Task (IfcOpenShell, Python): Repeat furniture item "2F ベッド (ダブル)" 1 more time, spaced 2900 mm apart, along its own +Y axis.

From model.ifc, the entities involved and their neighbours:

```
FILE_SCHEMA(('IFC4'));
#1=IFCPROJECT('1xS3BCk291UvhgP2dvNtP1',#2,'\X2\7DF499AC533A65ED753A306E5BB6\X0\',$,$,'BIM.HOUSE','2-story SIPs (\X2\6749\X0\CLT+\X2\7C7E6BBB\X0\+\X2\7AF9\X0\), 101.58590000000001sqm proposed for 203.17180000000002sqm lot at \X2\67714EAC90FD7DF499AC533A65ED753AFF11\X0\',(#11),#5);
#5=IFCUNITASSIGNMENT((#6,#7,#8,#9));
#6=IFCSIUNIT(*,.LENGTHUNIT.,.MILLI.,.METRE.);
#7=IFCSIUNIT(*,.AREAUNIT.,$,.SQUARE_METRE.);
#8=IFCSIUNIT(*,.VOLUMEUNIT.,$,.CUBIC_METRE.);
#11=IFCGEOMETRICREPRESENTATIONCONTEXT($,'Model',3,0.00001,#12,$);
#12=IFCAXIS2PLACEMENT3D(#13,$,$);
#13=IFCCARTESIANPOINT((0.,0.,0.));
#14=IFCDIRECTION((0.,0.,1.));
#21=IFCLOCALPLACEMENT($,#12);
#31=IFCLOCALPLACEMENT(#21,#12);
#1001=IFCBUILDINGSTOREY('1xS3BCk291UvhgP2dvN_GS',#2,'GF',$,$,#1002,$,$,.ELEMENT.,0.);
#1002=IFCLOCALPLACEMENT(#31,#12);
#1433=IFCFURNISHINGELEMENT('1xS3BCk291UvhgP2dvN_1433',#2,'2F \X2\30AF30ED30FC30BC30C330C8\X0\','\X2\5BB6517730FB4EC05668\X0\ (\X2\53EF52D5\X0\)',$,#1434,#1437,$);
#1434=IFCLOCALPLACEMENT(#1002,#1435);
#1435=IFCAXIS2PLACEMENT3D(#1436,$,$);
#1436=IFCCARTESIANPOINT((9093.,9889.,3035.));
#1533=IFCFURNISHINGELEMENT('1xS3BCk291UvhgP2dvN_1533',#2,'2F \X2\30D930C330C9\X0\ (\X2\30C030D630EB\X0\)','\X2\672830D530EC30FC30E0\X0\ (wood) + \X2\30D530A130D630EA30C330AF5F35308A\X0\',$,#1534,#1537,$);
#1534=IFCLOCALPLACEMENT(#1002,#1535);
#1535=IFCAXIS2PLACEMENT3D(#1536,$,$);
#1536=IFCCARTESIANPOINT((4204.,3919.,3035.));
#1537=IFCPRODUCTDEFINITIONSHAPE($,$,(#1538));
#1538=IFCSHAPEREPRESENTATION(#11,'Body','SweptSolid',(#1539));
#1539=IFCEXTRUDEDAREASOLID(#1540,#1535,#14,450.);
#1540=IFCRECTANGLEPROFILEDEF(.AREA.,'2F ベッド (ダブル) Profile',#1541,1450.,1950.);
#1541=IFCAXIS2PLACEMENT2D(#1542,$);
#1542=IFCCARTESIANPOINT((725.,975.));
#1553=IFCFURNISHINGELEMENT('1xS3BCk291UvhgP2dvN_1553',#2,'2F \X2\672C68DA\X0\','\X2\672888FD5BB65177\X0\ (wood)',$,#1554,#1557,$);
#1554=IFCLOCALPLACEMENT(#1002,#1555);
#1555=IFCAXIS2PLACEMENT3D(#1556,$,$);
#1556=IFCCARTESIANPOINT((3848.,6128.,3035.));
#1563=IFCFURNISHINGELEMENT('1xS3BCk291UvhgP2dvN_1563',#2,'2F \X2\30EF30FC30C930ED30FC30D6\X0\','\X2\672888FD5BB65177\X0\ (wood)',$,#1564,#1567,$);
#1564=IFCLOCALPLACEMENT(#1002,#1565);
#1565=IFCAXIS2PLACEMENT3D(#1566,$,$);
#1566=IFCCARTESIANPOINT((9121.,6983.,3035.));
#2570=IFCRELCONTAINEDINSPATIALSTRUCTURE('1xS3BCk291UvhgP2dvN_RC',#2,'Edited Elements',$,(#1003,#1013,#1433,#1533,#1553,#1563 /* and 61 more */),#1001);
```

```python
import ifcopenshell
import ifcopenshell.api.geometry
import ifcopenshell.api.root
import ifcopenshell.util.element
import ifcopenshell.util.placement
import ifcopenshell.util.unit

model = ifcopenshell.open("model.ifc")
unit_scale = ifcopenshell.util.unit.calculate_unit_scale(model)


def reuse_history(source, copy):
    """copy_class also copies each property set's owner history, people and application; keep the originals."""
    for rel in copy.IsDefinedBy:
        if rel.is_a("IfcRelDefinesByProperties") and (history := rel.RelatingPropertyDefinition.OwnerHistory):
            rel.RelatingPropertyDefinition.OwnerHistory = source.OwnerHistory
            ifcopenshell.util.element.remove_deep2(model, history)


source = model.by_guid("1xS3BCk291UvhgP2dvN_1533")
base = ifcopenshell.util.placement.get_local_placement(source.ObjectPlacement)
step = base[:3, 1] * 2.9 / unit_scale

for i in range(1, 2):
    copy = ifcopenshell.api.root.copy_class(model, product=source)
    copy.Representation = ifcopenshell.util.element.copy_deep(
        model, source.Representation, exclude=["IfcGeometricRepresentationContext", "IfcRepresentationMap"]
    )
    reuse_history(source, copy)
    matrix = base.copy()
    matrix[:3, 3] += i * step
    print("added at", matrix[:3, 3].round(3) + 0.0)
    ifcopenshell.api.geometry.edit_object_placement(model, product=copy, matrix=matrix, is_si=False)

model.write("model_rev.ifc")
```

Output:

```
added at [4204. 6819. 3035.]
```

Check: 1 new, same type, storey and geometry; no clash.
